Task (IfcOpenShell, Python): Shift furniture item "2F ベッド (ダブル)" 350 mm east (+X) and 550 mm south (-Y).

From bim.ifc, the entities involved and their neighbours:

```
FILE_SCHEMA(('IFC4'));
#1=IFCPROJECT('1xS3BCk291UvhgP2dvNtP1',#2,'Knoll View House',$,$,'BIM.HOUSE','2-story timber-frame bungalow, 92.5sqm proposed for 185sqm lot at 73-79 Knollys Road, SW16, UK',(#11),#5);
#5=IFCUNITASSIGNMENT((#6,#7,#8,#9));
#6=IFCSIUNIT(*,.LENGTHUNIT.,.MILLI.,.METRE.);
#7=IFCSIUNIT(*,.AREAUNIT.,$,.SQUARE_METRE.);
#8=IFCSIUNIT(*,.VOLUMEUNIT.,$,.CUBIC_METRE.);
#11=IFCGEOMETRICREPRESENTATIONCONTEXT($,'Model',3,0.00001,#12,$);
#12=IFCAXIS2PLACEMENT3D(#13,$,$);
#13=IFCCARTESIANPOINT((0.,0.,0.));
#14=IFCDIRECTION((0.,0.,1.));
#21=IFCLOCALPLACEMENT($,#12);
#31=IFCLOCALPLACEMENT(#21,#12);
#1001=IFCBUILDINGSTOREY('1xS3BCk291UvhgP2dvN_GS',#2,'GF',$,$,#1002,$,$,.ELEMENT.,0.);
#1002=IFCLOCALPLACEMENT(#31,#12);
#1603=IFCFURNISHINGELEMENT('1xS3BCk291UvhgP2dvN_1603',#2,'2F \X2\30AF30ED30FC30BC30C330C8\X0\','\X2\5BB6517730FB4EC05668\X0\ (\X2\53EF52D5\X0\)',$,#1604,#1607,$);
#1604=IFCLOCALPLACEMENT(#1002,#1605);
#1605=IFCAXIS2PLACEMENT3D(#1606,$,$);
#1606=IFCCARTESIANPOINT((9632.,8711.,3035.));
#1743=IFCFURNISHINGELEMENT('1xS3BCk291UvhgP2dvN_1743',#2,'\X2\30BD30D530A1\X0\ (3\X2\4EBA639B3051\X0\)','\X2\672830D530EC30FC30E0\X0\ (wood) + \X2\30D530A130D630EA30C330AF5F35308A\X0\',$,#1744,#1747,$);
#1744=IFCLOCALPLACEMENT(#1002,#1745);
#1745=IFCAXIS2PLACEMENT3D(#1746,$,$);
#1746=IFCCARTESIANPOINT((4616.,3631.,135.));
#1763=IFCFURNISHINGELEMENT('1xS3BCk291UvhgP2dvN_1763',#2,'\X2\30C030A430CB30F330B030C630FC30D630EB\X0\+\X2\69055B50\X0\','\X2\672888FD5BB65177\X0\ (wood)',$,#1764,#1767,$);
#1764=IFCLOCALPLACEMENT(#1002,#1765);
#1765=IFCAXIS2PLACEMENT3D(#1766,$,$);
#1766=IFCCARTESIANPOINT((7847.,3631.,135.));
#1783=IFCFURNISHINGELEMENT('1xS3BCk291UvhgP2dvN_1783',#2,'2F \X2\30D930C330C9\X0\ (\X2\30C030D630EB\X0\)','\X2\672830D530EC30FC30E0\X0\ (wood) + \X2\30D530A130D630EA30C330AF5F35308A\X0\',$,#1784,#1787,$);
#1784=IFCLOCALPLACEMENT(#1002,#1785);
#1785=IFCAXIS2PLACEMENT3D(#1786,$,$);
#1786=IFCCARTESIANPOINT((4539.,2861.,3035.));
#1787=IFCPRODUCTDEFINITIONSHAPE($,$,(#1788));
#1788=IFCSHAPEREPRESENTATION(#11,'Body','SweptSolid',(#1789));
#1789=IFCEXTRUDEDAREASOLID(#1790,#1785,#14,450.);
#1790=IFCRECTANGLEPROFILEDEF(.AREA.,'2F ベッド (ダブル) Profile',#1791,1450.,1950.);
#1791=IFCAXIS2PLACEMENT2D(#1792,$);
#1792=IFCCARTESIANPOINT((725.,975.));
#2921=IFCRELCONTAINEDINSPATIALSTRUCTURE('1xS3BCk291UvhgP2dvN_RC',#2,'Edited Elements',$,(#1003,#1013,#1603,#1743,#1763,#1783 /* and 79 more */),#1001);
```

```python
import ifcopenshell
import ifcopenshell.api.geometry
import ifcopenshell.util.placement
import ifcopenshell.util.unit

model = ifcopenshell.open("bim.ifc")
unit_scale = ifcopenshell.util.unit.calculate_unit_scale(model)

item = model.by_id(1783)
matrix = ifcopenshell.util.placement.get_local_placement(item.ObjectPlacement)
matrix[0, 3] += 0.35 / unit_scale
matrix[1, 3] -= 0.55 / unit_scale
ifcopenshell.api.geometry.edit_object_placement(model, product=item, matrix=matrix, is_si=False)

print(ifcopenshell.util.placement.get_local_placement(item.ObjectPlacement).round(3) + 0.0)

model.write("bim-out.ifc")
```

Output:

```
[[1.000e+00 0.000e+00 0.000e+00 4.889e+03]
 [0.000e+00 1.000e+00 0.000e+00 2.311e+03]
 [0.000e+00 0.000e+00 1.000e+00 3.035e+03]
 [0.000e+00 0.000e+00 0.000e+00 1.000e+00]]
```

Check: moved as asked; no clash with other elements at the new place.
